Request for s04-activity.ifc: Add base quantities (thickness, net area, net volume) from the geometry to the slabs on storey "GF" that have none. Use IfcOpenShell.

First a look at what the model holds.

```python
import ifcopenshell
import ifcopenshell.util.element
import ifcopenshell.util.unit

model = ifcopenshell.open("s04-activity.ifc")
print(model.schema)
for unit_type in ("LENGTHUNIT", "AREAUNIT", "VOLUMEUNIT"):
    print(unit_type, ifcopenshell.util.unit.calculate_unit_scale(model, unit_type))
storey = next(s for s in model.by_type("IfcBuildingStorey") if s.Name == "GF")
slabs = [e for e in ifcopenshell.util.element.get_decomposition(storey) if e.is_a("IfcSlab")]
for e in sorted(slabs, key=lambda e: e.id()):
    print(e.id(), e.is_a(), e.Name, list(ifcopenshell.util.element.get_psets(e, qtos_only=True)), sep=" | ")
```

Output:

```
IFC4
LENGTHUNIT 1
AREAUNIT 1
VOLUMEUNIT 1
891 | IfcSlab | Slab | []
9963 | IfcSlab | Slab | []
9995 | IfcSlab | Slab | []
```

```python
import ifcopenshell
import ifcopenshell.api.pset
import ifcopenshell.geom
import ifcopenshell.util.element
import ifcopenshell.util.shape
import ifcopenshell.util.unit

model = ifcopenshell.open("s04-activity.ifc")
unit_scale = ifcopenshell.util.unit.calculate_unit_scale(model)
area_scale = ifcopenshell.util.unit.calculate_unit_scale(model, "AREAUNIT")
volume_scale = ifcopenshell.util.unit.calculate_unit_scale(model, "VOLUMEUNIT")
settings = ifcopenshell.geom.settings()

storey = next(s for s in model.by_type("IfcBuildingStorey") if s.Name == "GF")
slabs = [e for e in ifcopenshell.util.element.get_decomposition(storey) if e.is_a("IfcSlab")]

for e in sorted(slabs, key=lambda e: e.id()):
    if ifcopenshell.util.element.get_psets(e, qtos_only=True, should_inherit=False):
        continue
    # Geometry comes back in metres, in the element's own axes.
    shape = ifcopenshell.geom.create_shape(settings, e)
    values = {
        "Width": ifcopenshell.util.shape.get_z(shape.geometry) / unit_scale,
        "NetArea": ifcopenshell.util.shape.get_footprint_area(shape.geometry) / area_scale,
        "NetVolume": ifcopenshell.util.shape.get_volume(shape.geometry) / volume_scale,
    }
    qto = ifcopenshell.api.pset.add_qto(model, product=e, name="Qto_SlabBaseQuantities")
    ifcopenshell.api.pset.edit_qto(model, qto=qto, properties=values)
    print(e.id(), {k: round(v, 3) for k, v in values.items()})

model.write("s04-activity-out.ifc")
```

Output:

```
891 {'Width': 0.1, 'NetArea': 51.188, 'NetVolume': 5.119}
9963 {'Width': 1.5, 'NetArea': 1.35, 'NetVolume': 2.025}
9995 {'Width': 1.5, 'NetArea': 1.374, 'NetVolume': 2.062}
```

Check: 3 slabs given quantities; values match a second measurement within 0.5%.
